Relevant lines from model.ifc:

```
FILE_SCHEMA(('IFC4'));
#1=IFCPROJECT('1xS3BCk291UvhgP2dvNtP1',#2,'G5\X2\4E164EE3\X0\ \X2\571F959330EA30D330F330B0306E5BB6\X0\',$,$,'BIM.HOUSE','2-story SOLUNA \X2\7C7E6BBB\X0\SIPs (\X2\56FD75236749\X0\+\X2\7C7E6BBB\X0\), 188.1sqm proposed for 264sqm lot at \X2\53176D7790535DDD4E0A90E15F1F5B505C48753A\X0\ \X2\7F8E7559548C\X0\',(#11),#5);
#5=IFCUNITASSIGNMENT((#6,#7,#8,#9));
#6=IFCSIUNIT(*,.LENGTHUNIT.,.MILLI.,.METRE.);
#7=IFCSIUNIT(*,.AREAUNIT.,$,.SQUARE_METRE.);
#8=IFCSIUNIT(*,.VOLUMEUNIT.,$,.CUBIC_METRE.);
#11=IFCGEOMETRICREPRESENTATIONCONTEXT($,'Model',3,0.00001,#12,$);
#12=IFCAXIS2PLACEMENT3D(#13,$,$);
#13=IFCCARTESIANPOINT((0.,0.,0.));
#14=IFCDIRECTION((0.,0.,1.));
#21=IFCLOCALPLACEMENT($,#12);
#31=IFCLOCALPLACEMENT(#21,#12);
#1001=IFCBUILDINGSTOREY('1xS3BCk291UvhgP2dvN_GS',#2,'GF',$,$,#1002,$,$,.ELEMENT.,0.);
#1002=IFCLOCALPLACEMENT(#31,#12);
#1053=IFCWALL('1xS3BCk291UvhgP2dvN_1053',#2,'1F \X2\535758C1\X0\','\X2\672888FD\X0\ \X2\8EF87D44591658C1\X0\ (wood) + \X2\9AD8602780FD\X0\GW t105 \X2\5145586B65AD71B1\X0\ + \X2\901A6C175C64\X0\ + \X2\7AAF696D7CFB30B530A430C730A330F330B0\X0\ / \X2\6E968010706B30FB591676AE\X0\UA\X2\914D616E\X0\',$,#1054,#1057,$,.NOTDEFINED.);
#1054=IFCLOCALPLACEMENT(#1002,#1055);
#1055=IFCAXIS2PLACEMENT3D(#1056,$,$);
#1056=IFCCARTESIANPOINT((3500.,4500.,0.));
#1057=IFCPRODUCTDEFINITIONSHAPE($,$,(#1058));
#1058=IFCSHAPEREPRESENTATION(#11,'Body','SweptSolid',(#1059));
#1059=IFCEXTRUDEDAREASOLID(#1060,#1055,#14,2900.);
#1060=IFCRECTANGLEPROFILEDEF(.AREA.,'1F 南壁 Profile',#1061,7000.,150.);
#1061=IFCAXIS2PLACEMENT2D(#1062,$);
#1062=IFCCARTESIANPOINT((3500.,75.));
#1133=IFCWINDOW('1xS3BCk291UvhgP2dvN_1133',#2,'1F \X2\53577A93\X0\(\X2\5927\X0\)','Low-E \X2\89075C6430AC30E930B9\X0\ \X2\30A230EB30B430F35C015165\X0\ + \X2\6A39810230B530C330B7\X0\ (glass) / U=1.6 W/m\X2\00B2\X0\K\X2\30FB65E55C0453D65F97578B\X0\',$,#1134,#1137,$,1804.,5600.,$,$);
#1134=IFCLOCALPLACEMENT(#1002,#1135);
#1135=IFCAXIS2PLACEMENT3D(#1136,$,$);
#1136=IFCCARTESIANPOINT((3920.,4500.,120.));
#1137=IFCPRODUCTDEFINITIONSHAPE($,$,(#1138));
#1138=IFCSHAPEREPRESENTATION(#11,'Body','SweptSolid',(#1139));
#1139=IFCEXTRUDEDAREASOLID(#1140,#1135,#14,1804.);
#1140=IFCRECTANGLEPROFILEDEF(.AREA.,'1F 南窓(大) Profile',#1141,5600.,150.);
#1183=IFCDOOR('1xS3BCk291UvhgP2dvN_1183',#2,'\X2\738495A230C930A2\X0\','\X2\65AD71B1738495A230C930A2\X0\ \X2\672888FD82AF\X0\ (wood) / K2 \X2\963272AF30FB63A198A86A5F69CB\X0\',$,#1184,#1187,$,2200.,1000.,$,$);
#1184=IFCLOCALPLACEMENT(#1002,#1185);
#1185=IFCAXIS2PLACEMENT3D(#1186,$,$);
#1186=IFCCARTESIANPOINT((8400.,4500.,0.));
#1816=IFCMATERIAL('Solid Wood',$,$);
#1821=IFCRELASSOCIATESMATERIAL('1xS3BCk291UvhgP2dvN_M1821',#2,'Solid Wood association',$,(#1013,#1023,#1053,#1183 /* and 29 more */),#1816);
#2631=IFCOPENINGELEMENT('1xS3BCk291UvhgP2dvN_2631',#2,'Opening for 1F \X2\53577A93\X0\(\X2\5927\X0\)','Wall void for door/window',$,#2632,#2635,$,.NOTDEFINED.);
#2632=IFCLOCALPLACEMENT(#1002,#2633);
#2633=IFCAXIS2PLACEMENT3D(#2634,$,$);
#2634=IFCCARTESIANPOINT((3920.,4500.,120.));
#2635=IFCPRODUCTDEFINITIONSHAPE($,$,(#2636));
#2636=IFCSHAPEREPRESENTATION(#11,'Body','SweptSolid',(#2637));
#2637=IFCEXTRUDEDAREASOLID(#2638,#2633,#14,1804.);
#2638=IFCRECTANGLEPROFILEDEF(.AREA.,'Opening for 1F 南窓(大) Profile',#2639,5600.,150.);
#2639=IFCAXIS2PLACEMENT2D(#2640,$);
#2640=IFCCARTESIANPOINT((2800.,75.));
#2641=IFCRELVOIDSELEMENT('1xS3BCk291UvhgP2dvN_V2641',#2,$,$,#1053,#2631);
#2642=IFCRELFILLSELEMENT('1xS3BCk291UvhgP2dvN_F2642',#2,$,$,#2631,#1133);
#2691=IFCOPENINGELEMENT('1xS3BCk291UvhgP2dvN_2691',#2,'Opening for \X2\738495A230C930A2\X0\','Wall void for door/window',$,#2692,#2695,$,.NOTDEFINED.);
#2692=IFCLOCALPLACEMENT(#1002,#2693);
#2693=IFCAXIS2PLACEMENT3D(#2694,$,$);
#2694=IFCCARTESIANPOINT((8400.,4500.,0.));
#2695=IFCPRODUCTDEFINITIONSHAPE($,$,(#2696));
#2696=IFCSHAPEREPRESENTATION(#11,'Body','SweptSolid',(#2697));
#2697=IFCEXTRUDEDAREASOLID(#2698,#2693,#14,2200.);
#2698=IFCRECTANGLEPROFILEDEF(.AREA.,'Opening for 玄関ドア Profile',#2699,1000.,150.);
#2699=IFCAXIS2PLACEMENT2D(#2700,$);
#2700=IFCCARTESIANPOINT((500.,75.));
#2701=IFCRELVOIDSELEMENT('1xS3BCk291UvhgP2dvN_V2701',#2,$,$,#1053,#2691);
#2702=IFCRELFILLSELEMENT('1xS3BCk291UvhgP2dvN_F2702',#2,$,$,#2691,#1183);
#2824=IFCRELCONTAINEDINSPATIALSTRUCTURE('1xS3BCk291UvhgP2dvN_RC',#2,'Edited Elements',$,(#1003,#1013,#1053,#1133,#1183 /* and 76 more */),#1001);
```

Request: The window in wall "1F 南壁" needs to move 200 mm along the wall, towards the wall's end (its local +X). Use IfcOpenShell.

```python
import ifcopenshell
import ifcopenshell.api.geometry
import ifcopenshell.util.placement
import ifcopenshell.util.unit

model = ifcopenshell.open("model.ifc")
unit_scale = ifcopenshell.util.unit.calculate_unit_scale(model)

window = model.by_id(1133)
opening = window.FillsVoids[0].RelatingOpeningElement
wall = opening.VoidsElements[0].RelatingBuildingElement

wall_matrix = ifcopenshell.util.placement.get_local_placement(wall.ObjectPlacement)
shift = wall_matrix[:3, 0] * 0.2 / unit_scale
before = ifcopenshell.util.placement.get_local_placement(window.ObjectPlacement)[:3, 3].copy()

# The window is not placed relative to its opening, so move both.
for product in (opening, window):
    matrix = ifcopenshell.util.placement.get_local_placement(product.ObjectPlacement)
    matrix[:3, 3] += shift
    ifcopenshell.api.geometry.edit_object_placement(model, product=product, matrix=matrix, is_si=False)

after = ifcopenshell.util.placement.get_local_placement(window.ObjectPlacement)[:3, 3]
print("window moved by", (after - before).round(3) + 0.0)

model.write("model_updated.ifc")
```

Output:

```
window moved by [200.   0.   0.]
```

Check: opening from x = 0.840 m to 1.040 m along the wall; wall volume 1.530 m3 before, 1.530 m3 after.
